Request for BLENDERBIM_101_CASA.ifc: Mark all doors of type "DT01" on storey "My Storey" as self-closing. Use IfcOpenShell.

First a look at what the model holds.

```python
import ifcopenshell
import ifcopenshell.util.element

model = ifcopenshell.open("BLENDERBIM_101_CASA.ifc")
print(model.schema)
storey = next(s for s in model.by_type("IfcBuildingStorey") if s.Name == "My Storey")
doors = [e for e in ifcopenshell.util.element.get_decomposition(storey) if e.is_a("IfcDoor")]
seen = {}
for e in doors:
    element_type = ifcopenshell.util.element.get_type(e)
    key = (element_type.Name if element_type != e and element_type else None, ifcopenshell.util.element.get_pset(e, "Pset_DoorCommon", "SelfClosing"))
    seen[key] = seen.get(key, 0) + 1
for (name, value), count in sorted(seen.items(), key=str):
    print(count, "x", name, "|", value)
```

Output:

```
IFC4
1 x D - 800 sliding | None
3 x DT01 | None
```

```python
import ifcopenshell
import ifcopenshell.api.pset
import ifcopenshell.util.element

model = ifcopenshell.open("BLENDERBIM_101_CASA.ifc")

storey = next(s for s in model.by_type("IfcBuildingStorey") if s.Name == "My Storey")
doors = [e for e in ifcopenshell.util.element.get_decomposition(storey) if e.is_a("IfcDoor")]

count = 0
for e in doors:
    element_type = ifcopenshell.util.element.get_type(e)
    if element_type in (None, e) or element_type.Name != "DT01":
        continue
    # add_pset returns the element's existing set when there is one.
    pset = ifcopenshell.api.pset.add_pset(model, product=e, name="Pset_DoorCommon")
    ifcopenshell.api.pset.edit_pset(model, pset=pset, properties={"SelfClosing": True})
    count += 1

print(count, "doors updated")

model.write("BLENDERBIM_101_CASA_edited.ifc")
```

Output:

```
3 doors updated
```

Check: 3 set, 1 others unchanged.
